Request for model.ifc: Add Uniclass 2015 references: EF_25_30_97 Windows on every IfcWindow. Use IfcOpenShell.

First a look at what the model holds.

```python
import ifcopenshell

model = ifcopenshell.open("model.ifc")
print(model.schema)
print("classifications:", [c.Name for c in model.by_type("IfcClassification")])
for ifc_class in ("IfcDoor", "IfcRoof", "IfcStair", "IfcWall", "IfcWindow"):
    print(ifc_class, len(model.by_type(ifc_class)))
```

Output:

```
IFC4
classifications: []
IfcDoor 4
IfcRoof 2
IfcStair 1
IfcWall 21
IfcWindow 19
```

```python
import ifcopenshell
import ifcopenshell.api.classification

model = ifcopenshell.open("model.ifc")

system = ifcopenshell.api.classification.add_classification(model, classification="Uniclass 2015")

codes = {
    "IfcWindow": ("EF_25_30_97", "Windows"),
}
for ifc_class, (code, name) in codes.items():
    products = model.by_type(ifc_class)
    ifcopenshell.api.classification.add_reference(
        model, products=products, classification=system, identification=code, name=name
    )
    print(code, len(products))

model.write("model-out.ifc")
```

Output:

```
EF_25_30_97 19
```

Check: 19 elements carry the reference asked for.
